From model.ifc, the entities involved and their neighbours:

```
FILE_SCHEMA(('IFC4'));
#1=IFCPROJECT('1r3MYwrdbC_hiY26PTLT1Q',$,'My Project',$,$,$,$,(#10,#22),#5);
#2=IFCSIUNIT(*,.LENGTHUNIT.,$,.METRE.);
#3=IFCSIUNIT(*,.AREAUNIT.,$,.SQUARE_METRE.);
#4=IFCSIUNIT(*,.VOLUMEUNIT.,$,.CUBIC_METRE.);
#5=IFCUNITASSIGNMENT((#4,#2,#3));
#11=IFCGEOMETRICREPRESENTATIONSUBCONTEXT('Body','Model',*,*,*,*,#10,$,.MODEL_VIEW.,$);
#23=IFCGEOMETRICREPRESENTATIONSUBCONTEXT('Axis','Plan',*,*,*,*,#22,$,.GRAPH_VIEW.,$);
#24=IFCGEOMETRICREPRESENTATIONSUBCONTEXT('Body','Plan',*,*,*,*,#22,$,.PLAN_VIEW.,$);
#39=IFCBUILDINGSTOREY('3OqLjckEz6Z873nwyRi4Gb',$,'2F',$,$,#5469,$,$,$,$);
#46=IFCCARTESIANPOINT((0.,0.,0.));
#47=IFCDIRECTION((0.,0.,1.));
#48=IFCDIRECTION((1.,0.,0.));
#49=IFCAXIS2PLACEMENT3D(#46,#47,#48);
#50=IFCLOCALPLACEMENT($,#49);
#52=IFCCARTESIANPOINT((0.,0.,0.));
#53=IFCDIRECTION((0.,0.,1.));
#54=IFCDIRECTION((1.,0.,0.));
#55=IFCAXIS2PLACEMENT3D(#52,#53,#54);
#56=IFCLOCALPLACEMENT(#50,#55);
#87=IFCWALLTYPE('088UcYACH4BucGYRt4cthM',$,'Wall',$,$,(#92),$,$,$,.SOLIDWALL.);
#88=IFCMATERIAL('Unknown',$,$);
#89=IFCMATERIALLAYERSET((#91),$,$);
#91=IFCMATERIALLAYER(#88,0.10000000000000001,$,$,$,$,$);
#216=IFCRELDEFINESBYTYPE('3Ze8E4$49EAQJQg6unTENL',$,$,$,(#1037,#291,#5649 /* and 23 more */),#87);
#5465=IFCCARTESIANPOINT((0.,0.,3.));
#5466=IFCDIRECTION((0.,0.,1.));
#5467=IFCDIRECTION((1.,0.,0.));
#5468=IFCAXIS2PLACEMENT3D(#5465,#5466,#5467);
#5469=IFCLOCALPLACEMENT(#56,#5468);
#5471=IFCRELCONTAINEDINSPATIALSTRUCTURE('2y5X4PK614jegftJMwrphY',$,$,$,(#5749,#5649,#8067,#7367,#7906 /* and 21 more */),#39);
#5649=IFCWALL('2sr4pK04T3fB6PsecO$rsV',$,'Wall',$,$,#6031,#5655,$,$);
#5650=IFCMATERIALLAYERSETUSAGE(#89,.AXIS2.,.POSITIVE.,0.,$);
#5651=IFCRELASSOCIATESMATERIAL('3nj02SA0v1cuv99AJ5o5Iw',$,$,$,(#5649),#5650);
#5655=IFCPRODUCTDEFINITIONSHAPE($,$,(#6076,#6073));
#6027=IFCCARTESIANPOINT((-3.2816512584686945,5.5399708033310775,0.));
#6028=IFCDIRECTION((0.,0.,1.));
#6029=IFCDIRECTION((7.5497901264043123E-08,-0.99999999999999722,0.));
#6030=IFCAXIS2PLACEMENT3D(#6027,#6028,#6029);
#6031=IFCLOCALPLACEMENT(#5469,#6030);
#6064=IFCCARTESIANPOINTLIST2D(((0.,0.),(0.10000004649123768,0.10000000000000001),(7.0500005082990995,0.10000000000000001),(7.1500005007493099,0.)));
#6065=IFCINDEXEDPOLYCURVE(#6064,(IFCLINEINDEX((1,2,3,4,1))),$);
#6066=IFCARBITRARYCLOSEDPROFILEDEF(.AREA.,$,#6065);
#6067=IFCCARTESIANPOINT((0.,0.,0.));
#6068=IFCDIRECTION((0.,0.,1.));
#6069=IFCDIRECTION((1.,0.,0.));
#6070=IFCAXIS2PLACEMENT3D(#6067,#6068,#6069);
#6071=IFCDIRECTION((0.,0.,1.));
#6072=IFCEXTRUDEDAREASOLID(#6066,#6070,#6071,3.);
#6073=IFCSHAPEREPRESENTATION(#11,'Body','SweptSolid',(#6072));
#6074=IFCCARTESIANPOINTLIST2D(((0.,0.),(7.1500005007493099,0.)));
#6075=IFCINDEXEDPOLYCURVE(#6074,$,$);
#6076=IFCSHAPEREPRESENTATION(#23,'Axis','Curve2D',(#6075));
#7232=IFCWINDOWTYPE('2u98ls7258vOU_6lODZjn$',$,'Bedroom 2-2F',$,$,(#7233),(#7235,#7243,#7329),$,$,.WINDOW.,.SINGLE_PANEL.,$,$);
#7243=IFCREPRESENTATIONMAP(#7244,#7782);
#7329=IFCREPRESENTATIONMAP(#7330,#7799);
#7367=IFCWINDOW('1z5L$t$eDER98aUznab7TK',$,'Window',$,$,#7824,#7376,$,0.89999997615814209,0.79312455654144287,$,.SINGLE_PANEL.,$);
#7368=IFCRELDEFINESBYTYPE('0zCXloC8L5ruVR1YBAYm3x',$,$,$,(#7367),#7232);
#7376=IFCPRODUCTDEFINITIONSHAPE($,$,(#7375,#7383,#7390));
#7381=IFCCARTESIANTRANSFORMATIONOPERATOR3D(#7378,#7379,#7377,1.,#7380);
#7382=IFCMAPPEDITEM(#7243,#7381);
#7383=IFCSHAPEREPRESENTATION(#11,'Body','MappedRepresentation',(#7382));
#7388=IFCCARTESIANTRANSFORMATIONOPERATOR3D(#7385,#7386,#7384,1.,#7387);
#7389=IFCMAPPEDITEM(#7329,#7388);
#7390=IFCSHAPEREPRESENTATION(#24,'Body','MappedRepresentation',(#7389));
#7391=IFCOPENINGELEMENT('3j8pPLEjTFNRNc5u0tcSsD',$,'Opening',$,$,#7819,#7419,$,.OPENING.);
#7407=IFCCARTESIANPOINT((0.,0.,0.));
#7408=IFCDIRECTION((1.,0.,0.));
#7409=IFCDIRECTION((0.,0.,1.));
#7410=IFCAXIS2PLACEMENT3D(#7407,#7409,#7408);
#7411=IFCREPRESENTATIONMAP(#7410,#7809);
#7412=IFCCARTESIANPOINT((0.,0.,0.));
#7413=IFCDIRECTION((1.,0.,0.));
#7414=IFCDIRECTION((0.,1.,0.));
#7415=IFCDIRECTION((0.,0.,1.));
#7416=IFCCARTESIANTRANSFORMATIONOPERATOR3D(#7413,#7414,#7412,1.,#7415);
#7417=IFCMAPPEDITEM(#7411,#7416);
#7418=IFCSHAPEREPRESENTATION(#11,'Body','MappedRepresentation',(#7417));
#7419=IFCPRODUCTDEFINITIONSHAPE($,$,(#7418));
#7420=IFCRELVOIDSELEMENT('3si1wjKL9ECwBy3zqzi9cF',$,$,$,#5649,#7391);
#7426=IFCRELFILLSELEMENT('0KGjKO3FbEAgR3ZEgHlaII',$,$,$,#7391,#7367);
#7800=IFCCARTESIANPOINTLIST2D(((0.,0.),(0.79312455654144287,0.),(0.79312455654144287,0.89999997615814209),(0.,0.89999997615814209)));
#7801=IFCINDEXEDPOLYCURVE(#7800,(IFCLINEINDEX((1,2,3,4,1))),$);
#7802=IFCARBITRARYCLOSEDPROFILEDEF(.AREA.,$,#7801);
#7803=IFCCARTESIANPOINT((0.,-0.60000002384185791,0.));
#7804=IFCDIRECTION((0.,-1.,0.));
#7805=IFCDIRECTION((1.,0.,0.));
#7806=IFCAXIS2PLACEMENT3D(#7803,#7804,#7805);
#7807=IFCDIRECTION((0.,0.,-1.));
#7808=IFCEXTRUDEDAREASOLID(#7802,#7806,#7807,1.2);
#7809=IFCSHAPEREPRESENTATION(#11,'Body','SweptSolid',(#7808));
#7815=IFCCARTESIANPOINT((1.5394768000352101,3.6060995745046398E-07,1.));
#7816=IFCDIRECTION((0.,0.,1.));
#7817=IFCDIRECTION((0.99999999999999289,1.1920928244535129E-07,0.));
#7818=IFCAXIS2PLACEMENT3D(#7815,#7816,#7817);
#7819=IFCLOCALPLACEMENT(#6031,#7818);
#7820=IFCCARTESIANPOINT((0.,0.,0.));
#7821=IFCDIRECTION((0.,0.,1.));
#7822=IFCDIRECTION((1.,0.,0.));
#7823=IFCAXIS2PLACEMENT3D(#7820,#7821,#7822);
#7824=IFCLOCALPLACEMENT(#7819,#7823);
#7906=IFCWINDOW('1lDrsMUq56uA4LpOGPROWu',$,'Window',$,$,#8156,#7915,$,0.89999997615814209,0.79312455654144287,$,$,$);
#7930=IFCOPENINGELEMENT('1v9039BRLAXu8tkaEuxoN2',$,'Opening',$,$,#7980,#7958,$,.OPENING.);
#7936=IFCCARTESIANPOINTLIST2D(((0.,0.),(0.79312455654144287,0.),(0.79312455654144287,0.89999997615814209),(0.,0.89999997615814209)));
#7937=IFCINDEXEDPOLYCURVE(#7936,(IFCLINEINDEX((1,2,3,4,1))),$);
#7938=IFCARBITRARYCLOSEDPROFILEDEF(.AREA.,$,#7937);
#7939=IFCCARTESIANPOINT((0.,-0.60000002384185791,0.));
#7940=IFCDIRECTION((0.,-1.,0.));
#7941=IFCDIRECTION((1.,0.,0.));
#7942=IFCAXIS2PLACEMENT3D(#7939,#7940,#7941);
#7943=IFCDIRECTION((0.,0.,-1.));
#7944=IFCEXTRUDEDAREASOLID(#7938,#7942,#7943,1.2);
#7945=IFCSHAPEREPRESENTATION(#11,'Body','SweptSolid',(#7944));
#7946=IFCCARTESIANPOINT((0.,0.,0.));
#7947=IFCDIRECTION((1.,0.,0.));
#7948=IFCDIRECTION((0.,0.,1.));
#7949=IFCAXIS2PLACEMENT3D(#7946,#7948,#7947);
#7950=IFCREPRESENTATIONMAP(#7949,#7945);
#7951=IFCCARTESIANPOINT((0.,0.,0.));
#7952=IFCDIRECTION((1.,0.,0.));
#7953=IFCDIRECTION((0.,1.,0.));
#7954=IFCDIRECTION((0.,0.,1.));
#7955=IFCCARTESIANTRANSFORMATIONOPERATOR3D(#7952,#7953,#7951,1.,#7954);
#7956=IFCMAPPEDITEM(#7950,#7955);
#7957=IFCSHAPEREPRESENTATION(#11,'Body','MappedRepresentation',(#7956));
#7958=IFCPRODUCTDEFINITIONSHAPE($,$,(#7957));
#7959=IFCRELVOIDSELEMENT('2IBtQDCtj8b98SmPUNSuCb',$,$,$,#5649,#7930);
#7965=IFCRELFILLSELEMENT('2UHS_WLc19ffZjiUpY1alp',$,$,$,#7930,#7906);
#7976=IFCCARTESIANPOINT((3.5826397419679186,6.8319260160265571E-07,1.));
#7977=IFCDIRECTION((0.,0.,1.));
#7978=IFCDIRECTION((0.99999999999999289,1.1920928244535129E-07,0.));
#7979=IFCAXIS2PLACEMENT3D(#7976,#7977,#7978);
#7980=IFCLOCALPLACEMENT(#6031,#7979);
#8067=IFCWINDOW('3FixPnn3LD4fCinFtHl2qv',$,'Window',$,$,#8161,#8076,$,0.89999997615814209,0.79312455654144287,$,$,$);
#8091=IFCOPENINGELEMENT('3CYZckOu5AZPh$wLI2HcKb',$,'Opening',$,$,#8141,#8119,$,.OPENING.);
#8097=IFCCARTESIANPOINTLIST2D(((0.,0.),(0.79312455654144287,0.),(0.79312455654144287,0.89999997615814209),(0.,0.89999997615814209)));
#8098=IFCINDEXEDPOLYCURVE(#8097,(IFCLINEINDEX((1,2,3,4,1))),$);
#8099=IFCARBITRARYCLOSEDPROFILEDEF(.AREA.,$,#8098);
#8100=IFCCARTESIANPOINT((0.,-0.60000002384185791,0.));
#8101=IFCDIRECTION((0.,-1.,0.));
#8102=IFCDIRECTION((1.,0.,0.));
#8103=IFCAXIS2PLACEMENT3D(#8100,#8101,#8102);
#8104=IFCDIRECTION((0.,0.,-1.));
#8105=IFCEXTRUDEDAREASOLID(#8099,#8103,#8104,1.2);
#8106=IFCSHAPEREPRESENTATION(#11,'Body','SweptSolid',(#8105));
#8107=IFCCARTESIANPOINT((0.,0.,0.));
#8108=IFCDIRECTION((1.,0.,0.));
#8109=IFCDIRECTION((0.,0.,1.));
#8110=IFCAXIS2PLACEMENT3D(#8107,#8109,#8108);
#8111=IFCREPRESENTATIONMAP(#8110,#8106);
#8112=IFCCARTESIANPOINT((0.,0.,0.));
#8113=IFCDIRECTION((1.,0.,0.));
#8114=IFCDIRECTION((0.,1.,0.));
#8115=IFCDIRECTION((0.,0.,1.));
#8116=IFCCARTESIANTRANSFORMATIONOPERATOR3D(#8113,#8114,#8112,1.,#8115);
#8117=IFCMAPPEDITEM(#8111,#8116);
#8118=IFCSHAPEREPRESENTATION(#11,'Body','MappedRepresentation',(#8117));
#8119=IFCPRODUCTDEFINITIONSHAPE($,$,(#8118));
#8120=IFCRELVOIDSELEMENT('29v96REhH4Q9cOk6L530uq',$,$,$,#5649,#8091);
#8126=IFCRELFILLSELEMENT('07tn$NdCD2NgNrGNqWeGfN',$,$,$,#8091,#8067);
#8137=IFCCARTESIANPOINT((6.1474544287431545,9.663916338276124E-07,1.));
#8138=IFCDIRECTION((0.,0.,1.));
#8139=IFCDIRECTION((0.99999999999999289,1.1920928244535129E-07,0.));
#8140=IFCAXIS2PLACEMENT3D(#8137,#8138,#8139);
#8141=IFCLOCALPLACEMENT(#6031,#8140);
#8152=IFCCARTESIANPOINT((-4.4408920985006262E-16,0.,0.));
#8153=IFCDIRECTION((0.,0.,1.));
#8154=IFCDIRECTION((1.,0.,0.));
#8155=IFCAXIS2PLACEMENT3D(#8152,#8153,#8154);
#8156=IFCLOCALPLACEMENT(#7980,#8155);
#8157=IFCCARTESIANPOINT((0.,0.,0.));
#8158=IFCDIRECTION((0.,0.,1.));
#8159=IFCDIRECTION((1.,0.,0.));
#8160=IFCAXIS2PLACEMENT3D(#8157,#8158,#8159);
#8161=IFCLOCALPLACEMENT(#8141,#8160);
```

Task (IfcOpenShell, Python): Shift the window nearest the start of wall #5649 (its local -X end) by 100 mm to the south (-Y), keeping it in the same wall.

```python
import ifcopenshell
import ifcopenshell.api.geometry
import ifcopenshell.util.placement
import ifcopenshell.util.unit

model = ifcopenshell.open("model.ifc")
unit_scale = ifcopenshell.util.unit.calculate_unit_scale(model)

window = model.by_guid("1z5L$t$eDER98aUznab7TK")
opening = window.FillsVoids[0].RelatingOpeningElement
wall = opening.VoidsElements[0].RelatingBuildingElement

wall_matrix = ifcopenshell.util.placement.get_local_placement(wall.ObjectPlacement)
shift = wall_matrix[:3, 0] * 0.1 / unit_scale
before = ifcopenshell.util.placement.get_local_placement(window.ObjectPlacement)[:3, 3].copy()

# The window is placed relative to its opening, so it follows when the opening moves.
matrix = ifcopenshell.util.placement.get_local_placement(opening.ObjectPlacement)
matrix[:3, 3] += shift
ifcopenshell.api.geometry.edit_object_placement(
    model, product=opening, matrix=matrix, is_si=False, should_transform_children=True
)

after = ifcopenshell.util.placement.get_local_placement(window.ObjectPlacement)[:3, 3]
print("window moved by", (after - before).round(3) + 0.0)

model.write("model_updated.ifc")
```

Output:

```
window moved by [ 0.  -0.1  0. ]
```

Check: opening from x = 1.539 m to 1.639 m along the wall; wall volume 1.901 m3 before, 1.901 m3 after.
